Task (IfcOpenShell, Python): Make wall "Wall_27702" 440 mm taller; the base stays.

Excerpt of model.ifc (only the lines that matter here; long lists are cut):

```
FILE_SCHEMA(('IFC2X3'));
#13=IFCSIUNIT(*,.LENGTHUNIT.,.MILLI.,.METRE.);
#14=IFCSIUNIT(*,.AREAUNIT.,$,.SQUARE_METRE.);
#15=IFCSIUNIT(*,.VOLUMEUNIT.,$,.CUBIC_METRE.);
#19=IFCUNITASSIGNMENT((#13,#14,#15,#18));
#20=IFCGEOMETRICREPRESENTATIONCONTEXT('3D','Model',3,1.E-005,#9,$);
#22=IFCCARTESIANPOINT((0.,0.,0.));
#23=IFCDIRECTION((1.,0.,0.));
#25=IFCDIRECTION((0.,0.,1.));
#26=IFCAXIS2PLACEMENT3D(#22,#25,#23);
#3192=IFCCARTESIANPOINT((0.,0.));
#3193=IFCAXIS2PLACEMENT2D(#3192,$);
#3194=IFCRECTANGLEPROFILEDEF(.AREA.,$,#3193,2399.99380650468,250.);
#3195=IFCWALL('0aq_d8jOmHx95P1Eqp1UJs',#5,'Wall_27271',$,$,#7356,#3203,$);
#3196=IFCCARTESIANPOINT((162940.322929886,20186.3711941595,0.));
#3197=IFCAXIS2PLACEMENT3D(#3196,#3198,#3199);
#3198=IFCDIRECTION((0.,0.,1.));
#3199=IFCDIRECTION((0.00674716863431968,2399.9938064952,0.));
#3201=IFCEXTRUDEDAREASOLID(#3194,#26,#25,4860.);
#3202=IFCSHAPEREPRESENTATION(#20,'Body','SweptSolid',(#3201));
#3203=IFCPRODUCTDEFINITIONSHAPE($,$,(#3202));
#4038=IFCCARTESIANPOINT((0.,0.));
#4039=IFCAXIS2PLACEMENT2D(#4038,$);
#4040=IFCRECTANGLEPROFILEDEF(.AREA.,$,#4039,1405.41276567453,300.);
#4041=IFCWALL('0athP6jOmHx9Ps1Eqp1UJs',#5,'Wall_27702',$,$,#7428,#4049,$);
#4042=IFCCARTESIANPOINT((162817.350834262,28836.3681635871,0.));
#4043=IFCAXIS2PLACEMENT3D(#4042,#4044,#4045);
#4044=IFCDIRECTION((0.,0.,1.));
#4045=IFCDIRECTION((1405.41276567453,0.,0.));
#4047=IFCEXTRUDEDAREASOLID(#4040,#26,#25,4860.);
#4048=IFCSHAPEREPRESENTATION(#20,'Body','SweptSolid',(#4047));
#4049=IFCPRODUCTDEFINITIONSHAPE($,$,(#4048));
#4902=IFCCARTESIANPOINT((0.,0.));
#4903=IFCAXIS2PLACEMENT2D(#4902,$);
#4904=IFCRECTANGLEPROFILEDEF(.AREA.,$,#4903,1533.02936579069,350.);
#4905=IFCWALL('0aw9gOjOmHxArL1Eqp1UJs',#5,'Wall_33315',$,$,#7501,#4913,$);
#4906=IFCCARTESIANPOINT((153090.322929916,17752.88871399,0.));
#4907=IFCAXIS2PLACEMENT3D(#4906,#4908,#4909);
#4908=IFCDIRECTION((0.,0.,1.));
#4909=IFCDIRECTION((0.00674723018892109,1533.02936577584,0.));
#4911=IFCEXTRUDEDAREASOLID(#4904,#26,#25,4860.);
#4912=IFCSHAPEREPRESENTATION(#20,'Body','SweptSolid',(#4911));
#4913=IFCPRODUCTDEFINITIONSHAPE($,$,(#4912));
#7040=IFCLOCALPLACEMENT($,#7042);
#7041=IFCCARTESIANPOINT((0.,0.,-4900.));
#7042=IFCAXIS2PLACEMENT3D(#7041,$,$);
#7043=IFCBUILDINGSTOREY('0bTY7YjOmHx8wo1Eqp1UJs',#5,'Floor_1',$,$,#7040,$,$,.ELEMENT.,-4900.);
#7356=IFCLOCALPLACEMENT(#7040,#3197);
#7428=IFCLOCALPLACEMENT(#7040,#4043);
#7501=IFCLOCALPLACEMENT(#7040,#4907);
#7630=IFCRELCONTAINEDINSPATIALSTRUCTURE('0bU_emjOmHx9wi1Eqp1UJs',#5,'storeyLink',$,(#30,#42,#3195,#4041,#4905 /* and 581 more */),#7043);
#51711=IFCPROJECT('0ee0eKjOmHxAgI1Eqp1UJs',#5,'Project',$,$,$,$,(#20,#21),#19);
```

```python
import ifcopenshell
import ifcopenshell.geom
import ifcopenshell.util.shape
import ifcopenshell.util.unit

model = ifcopenshell.open("model.ifc")
unit_scale = ifcopenshell.util.unit.calculate_unit_scale(model)
settings = ifcopenshell.geom.settings()


def volume(element):
    """Net volume in cubic metres, openings subtracted."""
    shape = ifcopenshell.geom.create_shape(settings, element)
    return ifcopenshell.util.shape.get_volume(shape.geometry)


wall = model.by_guid("0athP6jOmHx9Ps1Eqp1UJs")
before = volume(wall)

body = next(r for r in wall.Representation.Representations if r.RepresentationIdentifier == "Body")
solid = body.Items[0]
old_height = solid.Depth
solid.Depth += 0.44 / unit_scale
after = volume(wall)

print(f"height {old_height:g} -> {solid.Depth:g}, volume {before:.3f} -> {after:.3f} m3")

model.write("model-out.ifc")
```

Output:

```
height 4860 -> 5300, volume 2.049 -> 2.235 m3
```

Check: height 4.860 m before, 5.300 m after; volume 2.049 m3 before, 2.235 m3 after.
